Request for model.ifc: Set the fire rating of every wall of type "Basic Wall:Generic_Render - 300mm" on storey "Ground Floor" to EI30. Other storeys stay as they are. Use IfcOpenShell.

First a look at what the model holds.

```python
import ifcopenshell
import ifcopenshell.util.element

model = ifcopenshell.open("model.ifc")
print(model.schema)
storey = next(s for s in model.by_type("IfcBuildingStorey") if s.Name == "Ground Floor")
walls = [e for e in ifcopenshell.util.element.get_decomposition(storey) if e.is_a("IfcWall")]
seen = {}
for e in walls:
    element_type = ifcopenshell.util.element.get_type(e)
    key = (element_type.Name if element_type != e and element_type else None, ifcopenshell.util.element.get_pset(e, "Pset_WallCommon", "FireRating"))
    seen[key] = seen.get(key, 0) + 1
for (name, value), count in sorted(seen.items(), key=str):
    print(count, "x", name, "|", value)
```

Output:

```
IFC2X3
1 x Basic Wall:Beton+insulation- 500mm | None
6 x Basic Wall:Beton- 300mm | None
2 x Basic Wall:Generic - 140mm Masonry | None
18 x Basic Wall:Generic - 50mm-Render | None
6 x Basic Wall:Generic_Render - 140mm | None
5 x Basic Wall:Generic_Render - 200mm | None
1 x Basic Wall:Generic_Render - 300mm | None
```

```python
import ifcopenshell
import ifcopenshell.api.pset
import ifcopenshell.util.element

model = ifcopenshell.open("model.ifc")

storey = next(s for s in model.by_type("IfcBuildingStorey") if s.Name == "Ground Floor")
walls = [e for e in ifcopenshell.util.element.get_decomposition(storey) if e.is_a("IfcWall")]

count = 0
for e in walls:
    element_type = ifcopenshell.util.element.get_type(e)
    if element_type in (None, e) or element_type.Name != "Basic Wall:Generic_Render - 300mm":
        continue
    # add_pset returns the element's existing set when there is one.
    pset = ifcopenshell.api.pset.add_pset(model, product=e, name="Pset_WallCommon")
    ifcopenshell.api.pset.edit_pset(model, pset=pset, properties={"FireRating": "EI30"})
    count += 1

print(count, "walls updated")

model.write("model_rev.ifc")
```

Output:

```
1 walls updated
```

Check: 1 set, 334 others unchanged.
